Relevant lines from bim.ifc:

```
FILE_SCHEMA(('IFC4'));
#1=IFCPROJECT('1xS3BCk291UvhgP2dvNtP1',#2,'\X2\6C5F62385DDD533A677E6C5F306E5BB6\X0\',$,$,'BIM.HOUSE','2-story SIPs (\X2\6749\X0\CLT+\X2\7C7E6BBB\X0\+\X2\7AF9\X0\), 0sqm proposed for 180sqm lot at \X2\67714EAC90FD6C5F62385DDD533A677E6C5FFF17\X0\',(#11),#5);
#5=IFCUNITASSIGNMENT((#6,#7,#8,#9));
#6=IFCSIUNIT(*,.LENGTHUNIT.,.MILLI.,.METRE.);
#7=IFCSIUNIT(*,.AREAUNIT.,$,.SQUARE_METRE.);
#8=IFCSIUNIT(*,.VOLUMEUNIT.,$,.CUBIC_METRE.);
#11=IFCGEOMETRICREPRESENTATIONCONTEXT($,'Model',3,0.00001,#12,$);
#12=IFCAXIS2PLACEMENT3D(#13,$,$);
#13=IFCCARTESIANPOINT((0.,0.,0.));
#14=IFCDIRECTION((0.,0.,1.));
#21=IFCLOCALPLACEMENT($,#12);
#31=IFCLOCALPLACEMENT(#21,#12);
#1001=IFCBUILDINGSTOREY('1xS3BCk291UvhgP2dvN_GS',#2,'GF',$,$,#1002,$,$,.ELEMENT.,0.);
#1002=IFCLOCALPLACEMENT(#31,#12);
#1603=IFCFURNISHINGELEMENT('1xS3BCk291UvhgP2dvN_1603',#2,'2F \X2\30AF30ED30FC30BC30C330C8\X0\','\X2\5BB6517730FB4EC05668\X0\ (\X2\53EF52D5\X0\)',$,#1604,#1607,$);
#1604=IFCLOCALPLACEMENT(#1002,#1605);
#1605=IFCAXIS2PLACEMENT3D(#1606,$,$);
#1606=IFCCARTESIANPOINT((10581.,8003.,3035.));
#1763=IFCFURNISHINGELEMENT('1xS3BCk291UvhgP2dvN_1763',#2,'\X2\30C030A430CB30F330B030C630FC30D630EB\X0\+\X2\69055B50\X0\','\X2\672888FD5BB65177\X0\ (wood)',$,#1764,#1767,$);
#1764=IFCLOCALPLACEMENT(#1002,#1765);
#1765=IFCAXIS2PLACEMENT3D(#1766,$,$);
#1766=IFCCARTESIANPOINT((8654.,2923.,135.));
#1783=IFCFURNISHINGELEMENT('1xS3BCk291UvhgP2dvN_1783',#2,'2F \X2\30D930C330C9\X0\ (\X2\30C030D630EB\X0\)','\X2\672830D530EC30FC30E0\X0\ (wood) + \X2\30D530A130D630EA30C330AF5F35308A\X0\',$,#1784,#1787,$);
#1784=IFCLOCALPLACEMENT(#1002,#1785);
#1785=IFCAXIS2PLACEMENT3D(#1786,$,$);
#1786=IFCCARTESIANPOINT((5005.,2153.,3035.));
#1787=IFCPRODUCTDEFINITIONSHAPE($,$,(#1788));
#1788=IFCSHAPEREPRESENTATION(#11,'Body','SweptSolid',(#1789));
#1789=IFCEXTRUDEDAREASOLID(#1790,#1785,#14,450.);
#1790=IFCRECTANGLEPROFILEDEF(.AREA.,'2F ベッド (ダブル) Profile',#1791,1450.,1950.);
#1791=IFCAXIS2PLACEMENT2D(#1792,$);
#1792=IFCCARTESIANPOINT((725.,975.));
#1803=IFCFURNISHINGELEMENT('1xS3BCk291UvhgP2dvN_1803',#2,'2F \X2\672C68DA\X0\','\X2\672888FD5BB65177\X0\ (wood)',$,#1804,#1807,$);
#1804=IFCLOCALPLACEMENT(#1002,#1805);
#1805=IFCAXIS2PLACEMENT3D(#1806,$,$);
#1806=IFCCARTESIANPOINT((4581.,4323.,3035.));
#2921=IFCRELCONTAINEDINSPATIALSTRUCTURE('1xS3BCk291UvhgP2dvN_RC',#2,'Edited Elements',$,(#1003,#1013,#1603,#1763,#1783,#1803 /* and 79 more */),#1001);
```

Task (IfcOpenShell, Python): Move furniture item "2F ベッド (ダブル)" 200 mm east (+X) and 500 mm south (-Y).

```python
import ifcopenshell
import ifcopenshell.api.geometry
import ifcopenshell.util.placement
import ifcopenshell.util.unit

model = ifcopenshell.open("bim.ifc")
unit_scale = ifcopenshell.util.unit.calculate_unit_scale(model)

item = model.by_guid("1xS3BCk291UvhgP2dvN_1783")
matrix = ifcopenshell.util.placement.get_local_placement(item.ObjectPlacement)
matrix[0, 3] += 0.2 / unit_scale
matrix[1, 3] -= 0.5 / unit_scale
ifcopenshell.api.geometry.edit_object_placement(model, product=item, matrix=matrix, is_si=False)

print(ifcopenshell.util.placement.get_local_placement(item.ObjectPlacement).round(3) + 0.0)

model.write("bim_updated.ifc")
```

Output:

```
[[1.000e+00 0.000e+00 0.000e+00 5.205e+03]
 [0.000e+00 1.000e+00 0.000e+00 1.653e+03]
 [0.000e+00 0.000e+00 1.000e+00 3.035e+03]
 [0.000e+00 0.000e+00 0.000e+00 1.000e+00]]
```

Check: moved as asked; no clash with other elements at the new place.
